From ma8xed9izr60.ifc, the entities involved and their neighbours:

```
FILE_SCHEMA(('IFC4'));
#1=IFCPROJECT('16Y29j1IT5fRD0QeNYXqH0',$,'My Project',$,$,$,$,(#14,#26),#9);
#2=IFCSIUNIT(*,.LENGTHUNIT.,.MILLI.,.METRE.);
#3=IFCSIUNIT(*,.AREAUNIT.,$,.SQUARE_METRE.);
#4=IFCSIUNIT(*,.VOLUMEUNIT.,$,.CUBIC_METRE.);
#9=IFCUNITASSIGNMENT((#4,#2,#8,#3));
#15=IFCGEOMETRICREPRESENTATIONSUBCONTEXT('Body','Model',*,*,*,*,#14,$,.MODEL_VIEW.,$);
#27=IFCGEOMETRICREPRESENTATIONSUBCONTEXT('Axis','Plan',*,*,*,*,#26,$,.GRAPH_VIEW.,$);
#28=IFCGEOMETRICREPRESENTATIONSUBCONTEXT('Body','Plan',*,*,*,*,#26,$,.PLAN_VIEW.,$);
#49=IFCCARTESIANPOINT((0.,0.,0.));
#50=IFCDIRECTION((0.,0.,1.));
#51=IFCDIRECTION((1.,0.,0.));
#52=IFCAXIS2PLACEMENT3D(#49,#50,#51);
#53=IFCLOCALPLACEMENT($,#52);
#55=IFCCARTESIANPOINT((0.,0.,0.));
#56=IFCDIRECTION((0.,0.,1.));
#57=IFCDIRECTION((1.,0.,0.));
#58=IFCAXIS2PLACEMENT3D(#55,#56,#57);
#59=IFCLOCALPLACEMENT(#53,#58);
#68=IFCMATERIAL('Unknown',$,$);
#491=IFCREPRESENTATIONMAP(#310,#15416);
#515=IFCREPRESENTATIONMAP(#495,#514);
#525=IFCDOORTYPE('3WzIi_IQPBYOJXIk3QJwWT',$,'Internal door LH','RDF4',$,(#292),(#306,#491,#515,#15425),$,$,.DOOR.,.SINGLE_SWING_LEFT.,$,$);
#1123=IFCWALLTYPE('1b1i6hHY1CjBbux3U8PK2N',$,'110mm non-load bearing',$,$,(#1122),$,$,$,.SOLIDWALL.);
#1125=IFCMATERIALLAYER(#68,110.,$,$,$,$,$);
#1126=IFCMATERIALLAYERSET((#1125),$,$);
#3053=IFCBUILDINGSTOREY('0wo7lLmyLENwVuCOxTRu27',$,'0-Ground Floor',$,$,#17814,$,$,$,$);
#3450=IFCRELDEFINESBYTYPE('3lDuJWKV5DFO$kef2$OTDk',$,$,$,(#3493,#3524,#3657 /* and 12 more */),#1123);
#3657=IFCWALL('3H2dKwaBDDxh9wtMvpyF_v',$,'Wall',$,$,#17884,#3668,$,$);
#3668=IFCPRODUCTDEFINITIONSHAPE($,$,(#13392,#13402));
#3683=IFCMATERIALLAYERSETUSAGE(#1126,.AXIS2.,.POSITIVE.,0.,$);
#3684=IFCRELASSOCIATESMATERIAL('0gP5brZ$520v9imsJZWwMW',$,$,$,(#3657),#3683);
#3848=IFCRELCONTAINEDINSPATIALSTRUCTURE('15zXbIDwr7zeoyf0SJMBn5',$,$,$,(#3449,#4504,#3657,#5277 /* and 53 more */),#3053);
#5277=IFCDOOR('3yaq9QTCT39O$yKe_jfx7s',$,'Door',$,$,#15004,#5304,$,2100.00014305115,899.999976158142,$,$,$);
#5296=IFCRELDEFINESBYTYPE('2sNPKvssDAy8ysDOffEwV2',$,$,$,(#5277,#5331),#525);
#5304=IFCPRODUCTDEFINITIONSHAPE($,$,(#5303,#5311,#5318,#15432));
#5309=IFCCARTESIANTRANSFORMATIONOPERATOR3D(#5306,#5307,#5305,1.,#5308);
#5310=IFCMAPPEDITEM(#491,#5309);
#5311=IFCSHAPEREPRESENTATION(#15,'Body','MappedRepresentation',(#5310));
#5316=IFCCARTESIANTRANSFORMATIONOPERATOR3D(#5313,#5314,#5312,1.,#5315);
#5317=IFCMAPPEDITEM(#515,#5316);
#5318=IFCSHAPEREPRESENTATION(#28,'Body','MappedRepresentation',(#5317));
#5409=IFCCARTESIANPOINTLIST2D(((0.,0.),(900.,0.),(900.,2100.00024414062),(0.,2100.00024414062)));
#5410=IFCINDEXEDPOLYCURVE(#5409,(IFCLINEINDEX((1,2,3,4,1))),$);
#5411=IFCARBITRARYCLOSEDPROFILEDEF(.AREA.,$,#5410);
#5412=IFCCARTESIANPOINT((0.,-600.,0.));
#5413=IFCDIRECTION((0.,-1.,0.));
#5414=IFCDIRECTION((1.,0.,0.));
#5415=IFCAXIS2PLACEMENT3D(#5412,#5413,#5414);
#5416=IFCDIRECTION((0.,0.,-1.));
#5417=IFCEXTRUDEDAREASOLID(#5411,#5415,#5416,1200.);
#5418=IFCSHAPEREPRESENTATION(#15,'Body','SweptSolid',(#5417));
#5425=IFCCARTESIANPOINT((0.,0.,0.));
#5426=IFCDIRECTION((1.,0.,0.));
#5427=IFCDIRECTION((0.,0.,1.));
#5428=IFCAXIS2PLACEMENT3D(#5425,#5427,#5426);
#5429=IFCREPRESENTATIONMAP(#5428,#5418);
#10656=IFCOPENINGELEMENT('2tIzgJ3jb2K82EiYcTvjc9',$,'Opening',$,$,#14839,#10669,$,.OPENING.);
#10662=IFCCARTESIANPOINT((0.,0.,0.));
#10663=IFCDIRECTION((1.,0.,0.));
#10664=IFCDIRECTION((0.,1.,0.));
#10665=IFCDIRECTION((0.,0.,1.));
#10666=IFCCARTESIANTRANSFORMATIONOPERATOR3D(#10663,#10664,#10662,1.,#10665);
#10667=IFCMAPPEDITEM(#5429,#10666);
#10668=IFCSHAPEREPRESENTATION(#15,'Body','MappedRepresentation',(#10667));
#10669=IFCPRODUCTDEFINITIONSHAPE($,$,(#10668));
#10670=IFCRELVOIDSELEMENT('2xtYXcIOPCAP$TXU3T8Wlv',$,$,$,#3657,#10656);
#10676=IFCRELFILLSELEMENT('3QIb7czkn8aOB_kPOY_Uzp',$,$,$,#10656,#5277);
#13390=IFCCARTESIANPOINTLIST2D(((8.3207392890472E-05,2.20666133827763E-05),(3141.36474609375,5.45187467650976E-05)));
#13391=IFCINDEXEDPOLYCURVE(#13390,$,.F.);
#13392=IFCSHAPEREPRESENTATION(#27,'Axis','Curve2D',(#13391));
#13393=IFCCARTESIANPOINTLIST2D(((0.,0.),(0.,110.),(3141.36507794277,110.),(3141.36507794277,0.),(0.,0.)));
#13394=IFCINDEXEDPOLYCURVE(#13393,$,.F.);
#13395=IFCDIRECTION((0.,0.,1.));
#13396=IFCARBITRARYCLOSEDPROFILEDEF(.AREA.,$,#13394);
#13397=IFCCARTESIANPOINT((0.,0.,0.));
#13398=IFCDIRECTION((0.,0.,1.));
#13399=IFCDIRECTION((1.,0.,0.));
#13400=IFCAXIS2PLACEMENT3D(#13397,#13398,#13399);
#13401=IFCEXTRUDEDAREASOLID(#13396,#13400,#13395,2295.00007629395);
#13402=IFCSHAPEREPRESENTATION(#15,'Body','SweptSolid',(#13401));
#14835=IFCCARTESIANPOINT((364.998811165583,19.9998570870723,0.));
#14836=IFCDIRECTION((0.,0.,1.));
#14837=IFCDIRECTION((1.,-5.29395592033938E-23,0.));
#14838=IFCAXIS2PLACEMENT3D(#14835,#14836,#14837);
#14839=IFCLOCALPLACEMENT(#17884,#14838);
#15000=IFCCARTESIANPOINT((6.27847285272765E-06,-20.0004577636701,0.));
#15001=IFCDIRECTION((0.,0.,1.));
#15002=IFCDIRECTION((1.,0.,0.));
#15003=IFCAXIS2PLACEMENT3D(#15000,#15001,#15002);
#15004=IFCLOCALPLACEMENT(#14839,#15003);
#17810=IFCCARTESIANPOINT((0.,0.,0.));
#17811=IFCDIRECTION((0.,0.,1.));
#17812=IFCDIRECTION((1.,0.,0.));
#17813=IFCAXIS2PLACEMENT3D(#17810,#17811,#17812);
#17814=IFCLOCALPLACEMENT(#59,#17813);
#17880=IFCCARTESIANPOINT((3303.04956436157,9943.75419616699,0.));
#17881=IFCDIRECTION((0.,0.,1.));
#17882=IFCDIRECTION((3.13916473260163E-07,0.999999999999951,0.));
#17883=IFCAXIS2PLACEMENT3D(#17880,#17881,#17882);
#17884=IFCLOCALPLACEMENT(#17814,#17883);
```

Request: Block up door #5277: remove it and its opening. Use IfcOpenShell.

```python
import ifcopenshell
import ifcopenshell.api.feature
import ifcopenshell.api.root
import ifcopenshell.geom
import ifcopenshell.util.shape

model = ifcopenshell.open("ma8xed9izr60.ifc")
settings = ifcopenshell.geom.settings()


def volume(element):
    """Net volume in cubic metres, openings subtracted."""
    shape = ifcopenshell.geom.create_shape(settings, element)
    return ifcopenshell.util.shape.get_volume(shape.geometry)


door = model.by_id(5277)
opening = door.FillsVoids[0].RelatingOpeningElement
wall = opening.VoidsElements[0].RelatingBuildingElement
before = volume(wall)

ifcopenshell.api.root.remove_product(model, product=door)
ifcopenshell.api.feature.remove_feature(model, feature=opening)

after = volume(wall)

print(f"wall volume {before:.3f} -> {after:.3f} m3")

model.write("ma8xed9izr60_updated.ifc")
```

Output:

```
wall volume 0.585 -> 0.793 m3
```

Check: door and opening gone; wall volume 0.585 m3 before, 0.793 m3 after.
